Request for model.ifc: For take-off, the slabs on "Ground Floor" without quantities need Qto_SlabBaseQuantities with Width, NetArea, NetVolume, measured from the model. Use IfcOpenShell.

First a look at what the model holds.

```python
import ifcopenshell
import ifcopenshell.util.element
import ifcopenshell.util.unit

model = ifcopenshell.open("model.ifc")
print(model.schema)
for unit_type in ("LENGTHUNIT", "AREAUNIT", "VOLUMEUNIT"):
    print(unit_type, ifcopenshell.util.unit.calculate_unit_scale(model, unit_type))
storey = next(s for s in model.by_type("IfcBuildingStorey") if s.Name == "Ground Floor")
slabs = [e for e in ifcopenshell.util.element.get_decomposition(storey) if e.is_a("IfcSlab")]
for e in sorted(slabs, key=lambda e: e.id()):
    print(e.id(), e.is_a(), e.Name, list(ifcopenshell.util.element.get_psets(e, qtos_only=True)), sep=" | ")
```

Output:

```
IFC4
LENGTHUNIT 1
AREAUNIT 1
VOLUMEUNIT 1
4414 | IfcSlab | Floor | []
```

```python
import ifcopenshell
import ifcopenshell.api.pset
import ifcopenshell.geom
import ifcopenshell.util.element
import ifcopenshell.util.shape
import ifcopenshell.util.unit

model = ifcopenshell.open("model.ifc")
unit_scale = ifcopenshell.util.unit.calculate_unit_scale(model)
area_scale = ifcopenshell.util.unit.calculate_unit_scale(model, "AREAUNIT")
volume_scale = ifcopenshell.util.unit.calculate_unit_scale(model, "VOLUMEUNIT")
settings = ifcopenshell.geom.settings()

storey = next(s for s in model.by_type("IfcBuildingStorey") if s.Name == "Ground Floor")
slabs = [e for e in ifcopenshell.util.element.get_decomposition(storey) if e.is_a("IfcSlab")]

for e in sorted(slabs, key=lambda e: e.id()):
    if ifcopenshell.util.element.get_psets(e, qtos_only=True, should_inherit=False):
        continue
    # Geometry comes back in metres, in the element's own axes.
    shape = ifcopenshell.geom.create_shape(settings, e)
    values = {
        "Width": ifcopenshell.util.shape.get_z(shape.geometry) / unit_scale,
        "NetArea": ifcopenshell.util.shape.get_footprint_area(shape.geometry) / area_scale,
        "NetVolume": ifcopenshell.util.shape.get_volume(shape.geometry) / volume_scale,
    }
    qto = ifcopenshell.api.pset.add_qto(model, product=e, name="Qto_SlabBaseQuantities")
    ifcopenshell.api.pset.edit_qto(model, qto=qto, properties=values)
    print(e.id(), {k: round(v, 3) for k, v in values.items()})

model.write("model_edited.ifc")
```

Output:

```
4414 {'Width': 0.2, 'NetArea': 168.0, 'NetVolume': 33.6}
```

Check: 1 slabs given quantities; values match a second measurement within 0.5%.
